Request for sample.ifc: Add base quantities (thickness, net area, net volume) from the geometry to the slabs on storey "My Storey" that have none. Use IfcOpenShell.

First a look at what the model holds.

```python
import ifcopenshell
import ifcopenshell.util.element
import ifcopenshell.util.unit

model = ifcopenshell.open("sample.ifc")
print(model.schema)
for unit_type in ("LENGTHUNIT", "AREAUNIT", "VOLUMEUNIT"):
    print(unit_type, ifcopenshell.util.unit.calculate_unit_scale(model, unit_type))
storey = next(s for s in model.by_type("IfcBuildingStorey") if s.Name == "My Storey")
slabs = [e for e in ifcopenshell.util.element.get_decomposition(storey) if e.is_a("IfcSlab")]
for e in sorted(slabs, key=lambda e: e.id()):
    print(e.id(), e.is_a(), e.Name, list(ifcopenshell.util.element.get_psets(e, qtos_only=True)), sep=" | ")
```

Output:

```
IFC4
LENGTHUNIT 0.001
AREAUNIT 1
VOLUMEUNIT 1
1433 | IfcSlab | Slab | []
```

```python
import ifcopenshell
import ifcopenshell.api.pset
import ifcopenshell.geom
import ifcopenshell.util.element
import ifcopenshell.util.shape
import ifcopenshell.util.unit

model = ifcopenshell.open("sample.ifc")
unit_scale = ifcopenshell.util.unit.calculate_unit_scale(model)
area_scale = ifcopenshell.util.unit.calculate_unit_scale(model, "AREAUNIT")
volume_scale = ifcopenshell.util.unit.calculate_unit_scale(model, "VOLUMEUNIT")
settings = ifcopenshell.geom.settings()

storey = next(s for s in model.by_type("IfcBuildingStorey") if s.Name == "My Storey")
slabs = [e for e in ifcopenshell.util.element.get_decomposition(storey) if e.is_a("IfcSlab")]

for e in sorted(slabs, key=lambda e: e.id()):
    if ifcopenshell.util.element.get_psets(e, qtos_only=True, should_inherit=False):
        continue
    # Geometry comes back in metres, in the element's own axes.
    shape = ifcopenshell.geom.create_shape(settings, e)
    values = {
        "Width": ifcopenshell.util.shape.get_z(shape.geometry) / unit_scale,
        "NetArea": ifcopenshell.util.shape.get_footprint_area(shape.geometry) / area_scale,
        "NetVolume": ifcopenshell.util.shape.get_volume(shape.geometry) / volume_scale,
    }
    qto = ifcopenshell.api.pset.add_qto(model, product=e, name="Qto_SlabBaseQuantities")
    ifcopenshell.api.pset.edit_qto(model, qto=qto, properties=values)
    print(e.id(), {k: round(v, 3) for k, v in values.items()})

model.write("sample-out.ifc")
```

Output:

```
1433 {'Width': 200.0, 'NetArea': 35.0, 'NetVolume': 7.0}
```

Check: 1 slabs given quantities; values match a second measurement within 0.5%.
